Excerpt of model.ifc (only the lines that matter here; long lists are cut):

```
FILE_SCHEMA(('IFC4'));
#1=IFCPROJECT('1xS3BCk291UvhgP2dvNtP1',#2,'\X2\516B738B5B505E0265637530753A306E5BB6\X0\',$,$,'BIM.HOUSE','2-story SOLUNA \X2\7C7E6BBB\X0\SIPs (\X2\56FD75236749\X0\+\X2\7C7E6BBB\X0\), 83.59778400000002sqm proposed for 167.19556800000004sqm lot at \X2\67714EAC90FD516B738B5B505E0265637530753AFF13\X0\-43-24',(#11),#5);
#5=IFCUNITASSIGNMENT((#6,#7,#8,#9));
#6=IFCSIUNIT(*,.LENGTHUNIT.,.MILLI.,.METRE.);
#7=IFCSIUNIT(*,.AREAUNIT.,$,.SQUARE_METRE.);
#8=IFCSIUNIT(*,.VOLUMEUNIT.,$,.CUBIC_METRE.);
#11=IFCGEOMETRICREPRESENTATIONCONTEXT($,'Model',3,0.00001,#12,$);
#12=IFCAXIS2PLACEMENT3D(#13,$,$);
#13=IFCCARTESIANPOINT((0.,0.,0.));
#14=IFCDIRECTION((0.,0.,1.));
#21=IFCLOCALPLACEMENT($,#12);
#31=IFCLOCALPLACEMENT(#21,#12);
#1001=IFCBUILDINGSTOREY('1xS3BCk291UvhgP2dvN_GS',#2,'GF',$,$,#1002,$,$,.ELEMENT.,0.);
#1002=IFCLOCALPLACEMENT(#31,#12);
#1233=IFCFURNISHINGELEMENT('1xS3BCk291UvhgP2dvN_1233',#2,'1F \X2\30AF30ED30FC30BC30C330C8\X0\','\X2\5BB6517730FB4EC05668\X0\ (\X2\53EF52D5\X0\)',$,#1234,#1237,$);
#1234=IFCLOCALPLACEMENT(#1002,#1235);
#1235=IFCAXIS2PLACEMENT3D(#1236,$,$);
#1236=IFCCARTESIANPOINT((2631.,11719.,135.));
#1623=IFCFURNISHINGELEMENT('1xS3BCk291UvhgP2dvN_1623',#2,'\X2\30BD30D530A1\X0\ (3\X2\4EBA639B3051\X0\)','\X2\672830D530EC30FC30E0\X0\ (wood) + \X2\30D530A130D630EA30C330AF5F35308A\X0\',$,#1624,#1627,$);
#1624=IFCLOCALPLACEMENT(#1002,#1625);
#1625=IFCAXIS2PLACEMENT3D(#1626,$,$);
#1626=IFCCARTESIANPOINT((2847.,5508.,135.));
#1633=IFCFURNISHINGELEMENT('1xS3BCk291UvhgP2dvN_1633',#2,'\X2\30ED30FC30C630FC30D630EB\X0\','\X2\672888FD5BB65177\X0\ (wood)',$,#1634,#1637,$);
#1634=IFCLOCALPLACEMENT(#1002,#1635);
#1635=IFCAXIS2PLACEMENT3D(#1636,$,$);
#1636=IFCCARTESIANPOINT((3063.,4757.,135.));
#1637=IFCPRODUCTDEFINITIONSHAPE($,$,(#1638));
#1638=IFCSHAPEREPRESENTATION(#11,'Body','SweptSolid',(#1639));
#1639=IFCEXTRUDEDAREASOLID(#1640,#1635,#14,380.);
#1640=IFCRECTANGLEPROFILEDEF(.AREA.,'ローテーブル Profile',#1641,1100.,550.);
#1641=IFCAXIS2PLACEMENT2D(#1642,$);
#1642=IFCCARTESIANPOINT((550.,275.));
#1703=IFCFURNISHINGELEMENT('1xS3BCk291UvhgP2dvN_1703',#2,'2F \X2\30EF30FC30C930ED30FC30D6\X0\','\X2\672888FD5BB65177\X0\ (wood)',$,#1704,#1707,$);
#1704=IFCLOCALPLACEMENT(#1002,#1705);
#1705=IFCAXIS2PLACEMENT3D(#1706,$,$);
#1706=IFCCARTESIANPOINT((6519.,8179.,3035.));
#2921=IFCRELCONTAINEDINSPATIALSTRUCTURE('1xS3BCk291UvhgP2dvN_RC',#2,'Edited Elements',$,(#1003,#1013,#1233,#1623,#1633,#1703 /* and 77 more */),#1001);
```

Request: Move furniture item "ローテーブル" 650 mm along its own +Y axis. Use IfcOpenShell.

```python
import ifcopenshell
import ifcopenshell.api.geometry
import ifcopenshell.util.placement
import ifcopenshell.util.unit

model = ifcopenshell.open("model.ifc")
unit_scale = ifcopenshell.util.unit.calculate_unit_scale(model)

item = model.by_guid("1xS3BCk291UvhgP2dvN_1633")
matrix = ifcopenshell.util.placement.get_local_placement(item.ObjectPlacement)
matrix[:3, 3] += matrix[:3, 1] * 0.65 / unit_scale
ifcopenshell.api.geometry.edit_object_placement(model, product=item, matrix=matrix, is_si=False)

print(ifcopenshell.util.placement.get_local_placement(item.ObjectPlacement).round(3) + 0.0)

model.write("model-out.ifc")
```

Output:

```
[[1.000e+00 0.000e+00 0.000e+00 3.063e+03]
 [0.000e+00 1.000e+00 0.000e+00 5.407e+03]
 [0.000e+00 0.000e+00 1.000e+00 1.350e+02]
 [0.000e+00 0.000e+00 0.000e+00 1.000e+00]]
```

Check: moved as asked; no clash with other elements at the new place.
